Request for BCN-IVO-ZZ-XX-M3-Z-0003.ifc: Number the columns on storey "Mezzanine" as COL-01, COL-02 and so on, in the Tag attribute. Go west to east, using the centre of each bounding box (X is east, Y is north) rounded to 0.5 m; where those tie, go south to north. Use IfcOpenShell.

First a look at what the model holds.

```python
import ifcopenshell
import ifcopenshell.util.element
import ifcopenshell.util.placement

model = ifcopenshell.open("BCN-IVO-ZZ-XX-M3-Z-0003.ifc")
print(model.schema)
storey = next(s for s in model.by_type("IfcBuildingStorey") if s.Name == "Mezzanine")
columns = [e for e in ifcopenshell.util.element.get_decomposition(storey) if e.is_a("IfcColumn")]
for e in sorted(columns, key=lambda e: e.id()):
    origin = ifcopenshell.util.placement.get_local_placement(e.ObjectPlacement)[:3, 3]
    print(e.id(), e.Tag, e.Name, origin.round(2) + 0.0, sep=" | ")
```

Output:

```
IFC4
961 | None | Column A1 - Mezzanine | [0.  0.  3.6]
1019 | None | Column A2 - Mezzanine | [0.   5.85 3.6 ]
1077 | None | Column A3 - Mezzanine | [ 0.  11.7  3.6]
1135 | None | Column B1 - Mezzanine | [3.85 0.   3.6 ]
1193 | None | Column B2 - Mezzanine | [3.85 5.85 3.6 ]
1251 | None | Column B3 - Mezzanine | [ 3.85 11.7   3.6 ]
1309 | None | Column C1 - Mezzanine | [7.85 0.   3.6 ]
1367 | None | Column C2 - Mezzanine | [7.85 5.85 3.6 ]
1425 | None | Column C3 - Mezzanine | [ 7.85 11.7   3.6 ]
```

```python
import ifcopenshell
import ifcopenshell.geom
import ifcopenshell.util.element
import ifcopenshell.util.shape

model = ifcopenshell.open("BCN-IVO-ZZ-XX-M3-Z-0003.ifc")
settings = ifcopenshell.geom.settings()
settings.set("use-world-coords", True)


def centre(element):
    shape = ifcopenshell.geom.create_shape(settings, element)
    return ifcopenshell.util.shape.get_bbox_centroid(shape.geometry)


storey = next(s for s in model.by_type("IfcBuildingStorey") if s.Name == "Mezzanine")
columns = [e for e in ifcopenshell.util.element.get_decomposition(storey) if e.is_a("IfcColumn")]

# Insertion points can sit at a corner or the storey origin, so sort by the geometry (in metres).
centres = {e: centre(e) for e in columns}
columns.sort(key=lambda e: (round(centres[e][0] / 0.5), centres[e][1]))

for i, e in enumerate(columns, start=1):
    number = f"COL-{i:02d}"
    e.Tag = number
    print(e.id(), number)

model.write("BCN-IVO-ZZ-XX-M3-Z-0003_rev.ifc")
```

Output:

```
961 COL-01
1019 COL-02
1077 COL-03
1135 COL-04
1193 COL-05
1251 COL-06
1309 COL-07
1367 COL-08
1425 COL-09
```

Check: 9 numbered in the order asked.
